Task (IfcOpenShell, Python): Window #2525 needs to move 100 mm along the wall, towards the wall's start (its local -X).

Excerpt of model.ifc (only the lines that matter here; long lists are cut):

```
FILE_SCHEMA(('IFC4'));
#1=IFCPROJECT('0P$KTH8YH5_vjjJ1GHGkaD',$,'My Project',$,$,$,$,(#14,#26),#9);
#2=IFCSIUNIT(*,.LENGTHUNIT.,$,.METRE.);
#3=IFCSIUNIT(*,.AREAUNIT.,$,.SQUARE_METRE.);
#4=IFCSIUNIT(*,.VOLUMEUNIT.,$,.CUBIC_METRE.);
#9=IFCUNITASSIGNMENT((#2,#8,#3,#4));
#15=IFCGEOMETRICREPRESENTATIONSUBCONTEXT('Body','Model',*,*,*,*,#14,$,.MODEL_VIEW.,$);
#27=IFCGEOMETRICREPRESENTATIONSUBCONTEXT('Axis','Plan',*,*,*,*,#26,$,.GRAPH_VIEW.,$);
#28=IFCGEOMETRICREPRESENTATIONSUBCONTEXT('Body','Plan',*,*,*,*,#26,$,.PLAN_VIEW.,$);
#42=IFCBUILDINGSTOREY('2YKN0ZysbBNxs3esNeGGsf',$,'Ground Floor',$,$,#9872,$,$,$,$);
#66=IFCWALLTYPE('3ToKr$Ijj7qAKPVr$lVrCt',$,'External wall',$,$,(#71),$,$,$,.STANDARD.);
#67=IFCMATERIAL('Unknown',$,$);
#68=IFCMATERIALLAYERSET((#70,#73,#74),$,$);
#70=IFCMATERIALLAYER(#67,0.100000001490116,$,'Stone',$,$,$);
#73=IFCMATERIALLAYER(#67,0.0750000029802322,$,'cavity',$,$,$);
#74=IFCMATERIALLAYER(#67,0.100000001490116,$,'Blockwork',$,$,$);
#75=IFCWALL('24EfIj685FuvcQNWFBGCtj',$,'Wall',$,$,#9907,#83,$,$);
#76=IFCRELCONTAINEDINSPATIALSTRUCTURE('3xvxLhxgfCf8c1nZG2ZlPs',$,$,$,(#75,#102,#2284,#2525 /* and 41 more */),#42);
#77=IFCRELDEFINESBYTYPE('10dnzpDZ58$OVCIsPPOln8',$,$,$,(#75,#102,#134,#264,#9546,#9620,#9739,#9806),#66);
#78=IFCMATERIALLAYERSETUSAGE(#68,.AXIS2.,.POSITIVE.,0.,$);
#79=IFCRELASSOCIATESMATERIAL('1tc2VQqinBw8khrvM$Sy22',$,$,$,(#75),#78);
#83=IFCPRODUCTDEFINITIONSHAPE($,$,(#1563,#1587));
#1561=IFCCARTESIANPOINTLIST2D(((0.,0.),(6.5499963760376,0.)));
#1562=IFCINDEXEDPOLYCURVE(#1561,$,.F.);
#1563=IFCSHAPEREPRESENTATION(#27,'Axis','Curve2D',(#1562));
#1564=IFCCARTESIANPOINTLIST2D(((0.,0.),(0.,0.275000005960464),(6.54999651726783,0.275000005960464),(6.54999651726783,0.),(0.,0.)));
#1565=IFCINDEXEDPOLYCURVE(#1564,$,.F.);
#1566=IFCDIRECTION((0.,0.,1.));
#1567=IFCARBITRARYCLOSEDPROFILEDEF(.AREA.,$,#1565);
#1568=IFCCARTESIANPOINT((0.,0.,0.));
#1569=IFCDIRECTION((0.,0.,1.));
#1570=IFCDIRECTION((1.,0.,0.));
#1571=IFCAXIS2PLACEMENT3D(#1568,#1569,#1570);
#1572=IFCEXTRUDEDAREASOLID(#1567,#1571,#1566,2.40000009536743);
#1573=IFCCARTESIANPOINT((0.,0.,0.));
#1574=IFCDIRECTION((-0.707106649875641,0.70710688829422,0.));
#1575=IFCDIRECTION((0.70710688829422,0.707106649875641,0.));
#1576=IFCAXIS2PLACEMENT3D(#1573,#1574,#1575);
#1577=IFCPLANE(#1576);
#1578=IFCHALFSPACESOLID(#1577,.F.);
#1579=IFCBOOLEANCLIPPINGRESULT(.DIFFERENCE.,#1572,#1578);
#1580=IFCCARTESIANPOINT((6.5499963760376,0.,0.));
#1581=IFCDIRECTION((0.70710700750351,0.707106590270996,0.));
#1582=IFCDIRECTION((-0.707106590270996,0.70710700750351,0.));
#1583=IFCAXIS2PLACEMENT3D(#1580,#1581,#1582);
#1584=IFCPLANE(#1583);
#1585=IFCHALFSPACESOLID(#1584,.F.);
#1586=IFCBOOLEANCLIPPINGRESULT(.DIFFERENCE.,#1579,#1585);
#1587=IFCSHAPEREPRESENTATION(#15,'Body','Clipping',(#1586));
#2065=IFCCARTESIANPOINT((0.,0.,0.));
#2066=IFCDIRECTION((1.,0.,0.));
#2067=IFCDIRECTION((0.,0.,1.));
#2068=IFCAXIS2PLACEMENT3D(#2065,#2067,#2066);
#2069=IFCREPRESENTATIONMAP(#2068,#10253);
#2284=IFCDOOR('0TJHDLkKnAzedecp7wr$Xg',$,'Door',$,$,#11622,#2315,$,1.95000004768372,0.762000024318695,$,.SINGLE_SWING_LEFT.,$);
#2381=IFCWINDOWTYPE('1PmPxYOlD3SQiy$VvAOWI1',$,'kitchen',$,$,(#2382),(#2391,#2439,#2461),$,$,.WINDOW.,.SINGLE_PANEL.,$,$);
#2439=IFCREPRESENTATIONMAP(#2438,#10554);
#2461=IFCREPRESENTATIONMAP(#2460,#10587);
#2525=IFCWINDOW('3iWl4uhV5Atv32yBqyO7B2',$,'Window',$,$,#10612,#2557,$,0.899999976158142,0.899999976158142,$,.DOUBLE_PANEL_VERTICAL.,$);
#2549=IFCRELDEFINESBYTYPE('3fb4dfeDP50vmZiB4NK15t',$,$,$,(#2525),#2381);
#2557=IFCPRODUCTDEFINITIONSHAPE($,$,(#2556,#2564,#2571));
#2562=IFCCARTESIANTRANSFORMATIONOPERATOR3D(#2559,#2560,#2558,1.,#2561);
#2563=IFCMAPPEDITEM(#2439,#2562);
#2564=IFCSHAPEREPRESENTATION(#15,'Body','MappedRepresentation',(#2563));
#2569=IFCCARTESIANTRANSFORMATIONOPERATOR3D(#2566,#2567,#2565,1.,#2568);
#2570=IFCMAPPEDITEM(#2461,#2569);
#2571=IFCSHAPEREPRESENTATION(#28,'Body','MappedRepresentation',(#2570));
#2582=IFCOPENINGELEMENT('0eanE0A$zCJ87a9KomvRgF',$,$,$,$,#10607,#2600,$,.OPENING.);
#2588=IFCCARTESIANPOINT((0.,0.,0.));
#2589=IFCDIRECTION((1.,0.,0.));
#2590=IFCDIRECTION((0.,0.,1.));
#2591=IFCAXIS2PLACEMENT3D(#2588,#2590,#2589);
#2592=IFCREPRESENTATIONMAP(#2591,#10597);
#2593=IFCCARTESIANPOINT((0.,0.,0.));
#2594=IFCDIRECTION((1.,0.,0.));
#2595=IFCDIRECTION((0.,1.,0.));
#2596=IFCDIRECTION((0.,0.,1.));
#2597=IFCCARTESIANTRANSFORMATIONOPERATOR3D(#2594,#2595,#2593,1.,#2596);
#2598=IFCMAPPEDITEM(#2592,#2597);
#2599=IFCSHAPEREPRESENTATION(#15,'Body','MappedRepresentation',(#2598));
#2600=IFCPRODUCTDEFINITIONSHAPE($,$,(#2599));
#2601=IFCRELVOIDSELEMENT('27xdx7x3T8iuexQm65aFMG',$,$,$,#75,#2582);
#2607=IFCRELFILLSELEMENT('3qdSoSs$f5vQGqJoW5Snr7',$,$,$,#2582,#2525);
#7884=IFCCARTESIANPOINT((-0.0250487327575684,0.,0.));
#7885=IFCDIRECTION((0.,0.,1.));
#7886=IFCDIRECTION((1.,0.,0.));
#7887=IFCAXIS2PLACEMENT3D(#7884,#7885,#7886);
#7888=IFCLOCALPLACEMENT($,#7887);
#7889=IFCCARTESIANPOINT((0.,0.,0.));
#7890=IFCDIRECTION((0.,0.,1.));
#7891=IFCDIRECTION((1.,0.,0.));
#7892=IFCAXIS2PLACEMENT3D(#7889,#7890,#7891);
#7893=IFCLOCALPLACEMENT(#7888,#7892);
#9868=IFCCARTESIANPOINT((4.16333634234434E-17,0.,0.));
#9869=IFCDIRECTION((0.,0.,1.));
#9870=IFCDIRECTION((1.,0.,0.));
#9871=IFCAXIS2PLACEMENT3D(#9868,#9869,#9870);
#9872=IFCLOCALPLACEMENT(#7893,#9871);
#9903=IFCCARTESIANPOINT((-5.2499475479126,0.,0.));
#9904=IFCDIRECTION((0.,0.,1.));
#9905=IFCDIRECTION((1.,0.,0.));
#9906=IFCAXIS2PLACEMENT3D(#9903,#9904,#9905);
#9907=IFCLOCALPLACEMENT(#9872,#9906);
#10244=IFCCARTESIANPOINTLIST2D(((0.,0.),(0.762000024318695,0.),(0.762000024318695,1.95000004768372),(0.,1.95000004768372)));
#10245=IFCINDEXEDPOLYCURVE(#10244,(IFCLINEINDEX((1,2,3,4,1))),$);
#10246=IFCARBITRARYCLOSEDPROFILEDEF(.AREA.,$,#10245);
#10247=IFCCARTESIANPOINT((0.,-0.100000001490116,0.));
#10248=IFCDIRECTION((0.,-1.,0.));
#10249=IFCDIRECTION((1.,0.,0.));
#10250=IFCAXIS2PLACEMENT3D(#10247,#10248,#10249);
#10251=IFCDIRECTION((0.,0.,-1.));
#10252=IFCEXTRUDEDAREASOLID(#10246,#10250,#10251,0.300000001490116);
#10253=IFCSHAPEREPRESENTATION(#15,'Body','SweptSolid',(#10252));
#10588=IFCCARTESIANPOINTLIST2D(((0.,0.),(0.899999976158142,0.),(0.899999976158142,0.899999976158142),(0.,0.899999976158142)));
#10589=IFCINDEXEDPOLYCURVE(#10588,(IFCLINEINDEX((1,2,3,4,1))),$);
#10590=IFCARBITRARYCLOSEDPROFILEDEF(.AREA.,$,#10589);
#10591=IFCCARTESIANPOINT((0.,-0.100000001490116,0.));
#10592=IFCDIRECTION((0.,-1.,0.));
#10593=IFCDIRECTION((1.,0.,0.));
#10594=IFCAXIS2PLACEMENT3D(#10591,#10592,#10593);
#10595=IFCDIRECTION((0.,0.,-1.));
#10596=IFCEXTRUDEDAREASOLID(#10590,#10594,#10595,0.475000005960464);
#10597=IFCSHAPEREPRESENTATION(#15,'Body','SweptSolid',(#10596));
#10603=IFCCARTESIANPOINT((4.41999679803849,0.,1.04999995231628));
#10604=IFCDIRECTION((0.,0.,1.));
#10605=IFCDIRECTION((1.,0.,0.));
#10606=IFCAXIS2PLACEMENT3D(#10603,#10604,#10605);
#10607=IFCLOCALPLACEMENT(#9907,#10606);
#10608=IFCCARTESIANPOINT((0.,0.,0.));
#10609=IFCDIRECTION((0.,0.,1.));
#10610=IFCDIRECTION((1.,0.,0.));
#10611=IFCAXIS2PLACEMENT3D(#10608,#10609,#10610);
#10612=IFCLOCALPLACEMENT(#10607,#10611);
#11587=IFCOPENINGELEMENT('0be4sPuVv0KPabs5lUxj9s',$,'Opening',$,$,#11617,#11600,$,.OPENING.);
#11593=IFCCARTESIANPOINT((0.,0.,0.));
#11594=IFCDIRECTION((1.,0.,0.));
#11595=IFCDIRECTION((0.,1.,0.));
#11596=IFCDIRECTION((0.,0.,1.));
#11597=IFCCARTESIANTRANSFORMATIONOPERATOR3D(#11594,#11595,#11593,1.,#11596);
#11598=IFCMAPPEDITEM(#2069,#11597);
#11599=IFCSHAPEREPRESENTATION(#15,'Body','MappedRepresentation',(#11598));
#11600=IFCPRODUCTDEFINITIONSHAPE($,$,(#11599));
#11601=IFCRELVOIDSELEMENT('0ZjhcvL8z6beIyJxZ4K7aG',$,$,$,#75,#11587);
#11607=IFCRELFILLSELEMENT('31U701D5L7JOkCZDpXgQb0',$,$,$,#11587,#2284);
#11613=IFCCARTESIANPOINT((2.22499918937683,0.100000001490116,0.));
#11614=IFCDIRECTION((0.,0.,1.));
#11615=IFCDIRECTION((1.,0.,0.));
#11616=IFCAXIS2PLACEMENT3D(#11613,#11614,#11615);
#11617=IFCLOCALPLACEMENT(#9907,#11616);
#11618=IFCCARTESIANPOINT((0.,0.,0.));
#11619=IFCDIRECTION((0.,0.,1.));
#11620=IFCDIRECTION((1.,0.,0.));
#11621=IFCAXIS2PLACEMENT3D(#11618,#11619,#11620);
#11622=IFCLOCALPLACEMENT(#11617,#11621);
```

```python
import ifcopenshell
import ifcopenshell.api.geometry
import ifcopenshell.util.placement

model = ifcopenshell.open("model.ifc")

window = model.by_guid("3iWl4uhV5Atv32yBqyO7B2")
opening = window.FillsVoids[0].RelatingOpeningElement
wall = opening.VoidsElements[0].RelatingBuildingElement

wall_matrix = ifcopenshell.util.placement.get_local_placement(wall.ObjectPlacement)
shift = wall_matrix[:3, 0] * -0.1
before = ifcopenshell.util.placement.get_local_placement(window.ObjectPlacement)[:3, 3].copy()

# The window is placed relative to its opening, so it follows when the opening moves.
matrix = ifcopenshell.util.placement.get_local_placement(opening.ObjectPlacement)
matrix[:3, 3] += shift
ifcopenshell.api.geometry.edit_object_placement(
    model, product=opening, matrix=matrix, is_si=False, should_transform_children=True
)

after = ifcopenshell.util.placement.get_local_placement(window.ObjectPlacement)[:3, 3]
print("window moved by", (after - before).round(3) + 0.0)

model.write("model_rev.ifc")
```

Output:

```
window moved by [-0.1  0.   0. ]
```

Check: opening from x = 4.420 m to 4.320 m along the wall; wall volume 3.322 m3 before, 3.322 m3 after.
